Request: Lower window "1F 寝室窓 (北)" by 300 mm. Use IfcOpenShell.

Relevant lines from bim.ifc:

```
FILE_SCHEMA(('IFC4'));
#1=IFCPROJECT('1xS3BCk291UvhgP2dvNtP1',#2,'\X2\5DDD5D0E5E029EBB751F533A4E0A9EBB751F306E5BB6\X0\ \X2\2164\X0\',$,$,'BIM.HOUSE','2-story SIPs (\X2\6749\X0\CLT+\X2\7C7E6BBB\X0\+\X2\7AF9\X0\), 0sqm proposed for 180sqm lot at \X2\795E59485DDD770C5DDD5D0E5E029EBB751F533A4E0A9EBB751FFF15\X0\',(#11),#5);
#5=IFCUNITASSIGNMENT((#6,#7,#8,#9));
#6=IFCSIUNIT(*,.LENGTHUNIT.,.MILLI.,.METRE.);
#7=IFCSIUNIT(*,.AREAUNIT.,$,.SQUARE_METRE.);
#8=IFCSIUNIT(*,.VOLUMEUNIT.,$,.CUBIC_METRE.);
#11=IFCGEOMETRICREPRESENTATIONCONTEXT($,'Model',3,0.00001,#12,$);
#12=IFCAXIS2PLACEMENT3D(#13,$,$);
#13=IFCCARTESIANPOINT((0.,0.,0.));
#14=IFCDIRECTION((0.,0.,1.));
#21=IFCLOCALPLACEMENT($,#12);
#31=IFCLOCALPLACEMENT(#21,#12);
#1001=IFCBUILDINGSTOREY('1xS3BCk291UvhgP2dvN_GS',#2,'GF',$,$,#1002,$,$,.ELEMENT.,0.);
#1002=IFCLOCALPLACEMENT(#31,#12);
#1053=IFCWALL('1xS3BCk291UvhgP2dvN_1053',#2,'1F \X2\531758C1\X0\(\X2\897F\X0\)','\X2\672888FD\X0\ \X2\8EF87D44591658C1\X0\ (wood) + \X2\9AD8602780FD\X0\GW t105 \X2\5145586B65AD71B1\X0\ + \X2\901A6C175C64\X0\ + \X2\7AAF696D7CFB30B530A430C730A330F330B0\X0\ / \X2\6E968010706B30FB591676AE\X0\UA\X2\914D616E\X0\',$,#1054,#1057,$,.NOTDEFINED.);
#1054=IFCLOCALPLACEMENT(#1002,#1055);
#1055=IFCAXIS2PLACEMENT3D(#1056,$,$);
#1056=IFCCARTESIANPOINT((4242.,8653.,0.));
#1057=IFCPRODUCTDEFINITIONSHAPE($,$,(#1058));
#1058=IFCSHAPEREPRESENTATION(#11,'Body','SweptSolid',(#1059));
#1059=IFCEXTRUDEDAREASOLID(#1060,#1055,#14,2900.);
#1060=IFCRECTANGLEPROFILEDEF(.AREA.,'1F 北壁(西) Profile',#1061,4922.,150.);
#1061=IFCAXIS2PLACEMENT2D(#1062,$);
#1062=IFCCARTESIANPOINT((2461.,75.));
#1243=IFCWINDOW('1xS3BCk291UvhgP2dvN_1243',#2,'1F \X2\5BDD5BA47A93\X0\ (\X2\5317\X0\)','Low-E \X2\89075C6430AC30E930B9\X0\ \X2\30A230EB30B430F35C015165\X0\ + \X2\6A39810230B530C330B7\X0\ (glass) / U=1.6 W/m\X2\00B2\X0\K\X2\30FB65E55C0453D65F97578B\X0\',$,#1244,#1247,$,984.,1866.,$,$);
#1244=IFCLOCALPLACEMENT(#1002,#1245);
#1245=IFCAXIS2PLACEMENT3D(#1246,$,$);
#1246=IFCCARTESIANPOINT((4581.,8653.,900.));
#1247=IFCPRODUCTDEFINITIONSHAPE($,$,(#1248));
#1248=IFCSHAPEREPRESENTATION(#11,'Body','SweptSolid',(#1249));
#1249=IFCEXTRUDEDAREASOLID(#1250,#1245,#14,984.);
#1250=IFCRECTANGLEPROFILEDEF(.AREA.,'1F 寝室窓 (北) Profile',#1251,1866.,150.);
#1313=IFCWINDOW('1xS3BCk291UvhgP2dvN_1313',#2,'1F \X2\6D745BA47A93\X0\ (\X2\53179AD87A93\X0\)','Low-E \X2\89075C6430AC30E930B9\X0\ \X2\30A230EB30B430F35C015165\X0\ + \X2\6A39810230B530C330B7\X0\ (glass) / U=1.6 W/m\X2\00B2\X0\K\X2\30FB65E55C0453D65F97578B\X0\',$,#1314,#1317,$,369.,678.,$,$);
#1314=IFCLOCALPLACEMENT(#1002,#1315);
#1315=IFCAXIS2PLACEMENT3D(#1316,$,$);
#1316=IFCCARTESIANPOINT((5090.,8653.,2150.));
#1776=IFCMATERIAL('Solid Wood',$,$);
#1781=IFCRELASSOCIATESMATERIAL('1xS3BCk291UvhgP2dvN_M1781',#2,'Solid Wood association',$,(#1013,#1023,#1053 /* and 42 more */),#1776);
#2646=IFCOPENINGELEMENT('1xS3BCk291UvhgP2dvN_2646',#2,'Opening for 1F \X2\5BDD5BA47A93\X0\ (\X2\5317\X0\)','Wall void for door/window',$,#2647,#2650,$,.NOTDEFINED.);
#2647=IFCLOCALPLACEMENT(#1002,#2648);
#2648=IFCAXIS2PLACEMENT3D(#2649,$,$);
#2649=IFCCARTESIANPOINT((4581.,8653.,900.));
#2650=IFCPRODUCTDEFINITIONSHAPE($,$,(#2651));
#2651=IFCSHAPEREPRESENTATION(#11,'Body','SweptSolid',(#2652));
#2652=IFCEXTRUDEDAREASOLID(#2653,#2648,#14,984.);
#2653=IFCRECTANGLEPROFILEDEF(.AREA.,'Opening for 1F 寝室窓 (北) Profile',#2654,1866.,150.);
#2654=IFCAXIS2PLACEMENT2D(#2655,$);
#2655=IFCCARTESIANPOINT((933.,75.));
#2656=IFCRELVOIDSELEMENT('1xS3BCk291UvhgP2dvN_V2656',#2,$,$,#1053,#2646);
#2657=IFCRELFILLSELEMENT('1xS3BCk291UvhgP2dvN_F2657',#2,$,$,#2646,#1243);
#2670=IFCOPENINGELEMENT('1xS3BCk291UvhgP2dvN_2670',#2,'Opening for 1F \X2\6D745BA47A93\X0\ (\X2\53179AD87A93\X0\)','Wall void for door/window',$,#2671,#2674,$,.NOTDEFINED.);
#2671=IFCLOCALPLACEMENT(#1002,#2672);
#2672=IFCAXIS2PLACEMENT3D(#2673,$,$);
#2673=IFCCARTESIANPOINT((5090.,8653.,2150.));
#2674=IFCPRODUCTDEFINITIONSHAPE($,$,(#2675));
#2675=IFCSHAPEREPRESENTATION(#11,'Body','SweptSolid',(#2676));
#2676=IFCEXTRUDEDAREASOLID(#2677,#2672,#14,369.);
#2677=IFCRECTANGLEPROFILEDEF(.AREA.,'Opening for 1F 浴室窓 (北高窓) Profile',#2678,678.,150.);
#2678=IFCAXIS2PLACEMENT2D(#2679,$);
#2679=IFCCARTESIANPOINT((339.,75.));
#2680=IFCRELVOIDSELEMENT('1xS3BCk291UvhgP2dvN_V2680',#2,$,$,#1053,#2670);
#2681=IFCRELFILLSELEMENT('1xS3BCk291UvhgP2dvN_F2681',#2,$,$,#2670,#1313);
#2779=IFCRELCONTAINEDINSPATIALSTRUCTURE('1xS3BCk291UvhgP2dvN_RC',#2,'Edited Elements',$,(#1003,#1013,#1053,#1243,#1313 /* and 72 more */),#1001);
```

```python
import numpy as np
import ifcopenshell
import ifcopenshell.api.geometry
import ifcopenshell.util.placement
import ifcopenshell.util.unit

model = ifcopenshell.open("bim.ifc")
unit_scale = ifcopenshell.util.unit.calculate_unit_scale(model)

window = model.by_id(1243)
opening = window.FillsVoids[0].RelatingOpeningElement
dz = -0.3 / unit_scale

shift = np.array([0.0, 0.0, dz])
# The window is not placed relative to its opening, so move both.
for product in (opening, window):
    matrix = ifcopenshell.util.placement.get_local_placement(product.ObjectPlacement)
    matrix[:3, 3] += shift
    ifcopenshell.api.geometry.edit_object_placement(model, product=product, matrix=matrix, is_si=False)

print(f"moved by {dz * unit_scale:+.3f} m")

model.write("bim_rev.ifc")
```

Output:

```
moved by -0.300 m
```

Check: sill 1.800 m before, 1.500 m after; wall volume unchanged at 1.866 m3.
